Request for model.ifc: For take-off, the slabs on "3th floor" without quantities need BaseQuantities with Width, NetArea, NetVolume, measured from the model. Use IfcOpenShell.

First a look at what the model holds.

```python
import ifcopenshell
import ifcopenshell.util.element
import ifcopenshell.util.unit

model = ifcopenshell.open("model.ifc")
print(model.schema)
for unit_type in ("LENGTHUNIT", "AREAUNIT", "VOLUMEUNIT"):
    print(unit_type, ifcopenshell.util.unit.calculate_unit_scale(model, unit_type))
storey = next(s for s in model.by_type("IfcBuildingStorey") if s.Name == "3th floor")
slabs = [e for e in ifcopenshell.util.element.get_decomposition(storey) if e.is_a("IfcSlab")]
for e in sorted(slabs, key=lambda e: e.id()):
    print(e.id(), e.is_a(), e.Name, list(ifcopenshell.util.element.get_psets(e, qtos_only=True)), sep=" | ")
```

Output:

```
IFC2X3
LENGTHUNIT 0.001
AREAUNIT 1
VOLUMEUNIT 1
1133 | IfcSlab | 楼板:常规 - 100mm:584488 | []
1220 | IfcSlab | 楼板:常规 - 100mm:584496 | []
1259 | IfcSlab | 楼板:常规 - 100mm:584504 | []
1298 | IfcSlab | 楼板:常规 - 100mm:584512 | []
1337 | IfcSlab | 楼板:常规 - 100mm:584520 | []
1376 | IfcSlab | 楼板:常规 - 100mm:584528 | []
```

```python
import ifcopenshell
import ifcopenshell.api.pset
import ifcopenshell.geom
import ifcopenshell.util.element
import ifcopenshell.util.shape
import ifcopenshell.util.unit

model = ifcopenshell.open("model.ifc")
unit_scale = ifcopenshell.util.unit.calculate_unit_scale(model)
area_scale = ifcopenshell.util.unit.calculate_unit_scale(model, "AREAUNIT")
volume_scale = ifcopenshell.util.unit.calculate_unit_scale(model, "VOLUMEUNIT")
settings = ifcopenshell.geom.settings()

storey = next(s for s in model.by_type("IfcBuildingStorey") if s.Name == "3th floor")
slabs = [e for e in ifcopenshell.util.element.get_decomposition(storey) if e.is_a("IfcSlab")]

for e in sorted(slabs, key=lambda e: e.id()):
    if ifcopenshell.util.element.get_psets(e, qtos_only=True, should_inherit=False):
        continue
    # Geometry comes back in metres, in the element's own axes.
    shape = ifcopenshell.geom.create_shape(settings, e)
    values = {
        "Width": ifcopenshell.util.shape.get_z(shape.geometry) / unit_scale,
        "NetArea": ifcopenshell.util.shape.get_footprint_area(shape.geometry) / area_scale,
        "NetVolume": ifcopenshell.util.shape.get_volume(shape.geometry) / volume_scale,
    }
    qto = ifcopenshell.api.pset.add_qto(model, product=e, name="BaseQuantities")
    ifcopenshell.api.pset.edit_qto(model, qto=qto, properties=values)
    print(e.id(), {k: round(v, 3) for k, v in values.items()})

model.write("model-out.ifc")
```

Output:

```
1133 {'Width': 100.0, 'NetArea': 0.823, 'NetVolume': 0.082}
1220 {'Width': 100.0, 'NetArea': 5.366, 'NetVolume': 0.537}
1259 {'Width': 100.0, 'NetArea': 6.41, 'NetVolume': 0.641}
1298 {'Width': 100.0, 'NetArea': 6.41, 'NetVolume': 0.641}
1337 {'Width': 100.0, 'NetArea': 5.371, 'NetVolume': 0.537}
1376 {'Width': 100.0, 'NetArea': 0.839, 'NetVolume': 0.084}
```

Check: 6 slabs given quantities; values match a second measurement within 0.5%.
